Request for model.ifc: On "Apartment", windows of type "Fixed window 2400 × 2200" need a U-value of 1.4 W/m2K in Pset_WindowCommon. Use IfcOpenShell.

First a look at what the model holds.

```python
import ifcopenshell
import ifcopenshell.util.element

model = ifcopenshell.open("model.ifc")
print(model.schema)
storey = next(s for s in model.by_type("IfcBuildingStorey") if s.Name == "Apartment")
windows = [e for e in ifcopenshell.util.element.get_decomposition(storey) if e.is_a("IfcWindow")]
seen = {}
for e in windows:
    element_type = ifcopenshell.util.element.get_type(e)
    key = (element_type.Name if element_type != e and element_type else None, ifcopenshell.util.element.get_pset(e, "Pset_WindowCommon", "ThermalTransmittance"))
    seen[key] = seen.get(key, 0) + 1
for (name, value), count in sorted(seen.items(), key=str):
    print(count, "x", name, "|", value)
```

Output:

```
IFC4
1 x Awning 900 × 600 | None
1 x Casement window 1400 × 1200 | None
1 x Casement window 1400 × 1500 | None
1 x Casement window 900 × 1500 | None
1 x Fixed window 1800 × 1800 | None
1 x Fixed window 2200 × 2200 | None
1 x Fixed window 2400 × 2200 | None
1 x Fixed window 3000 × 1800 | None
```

```python
import ifcopenshell
import ifcopenshell.api.pset
import ifcopenshell.util.element

model = ifcopenshell.open("model.ifc")

storey = next(s for s in model.by_type("IfcBuildingStorey") if s.Name == "Apartment")
windows = [e for e in ifcopenshell.util.element.get_decomposition(storey) if e.is_a("IfcWindow")]

count = 0
for e in windows:
    element_type = ifcopenshell.util.element.get_type(e)
    if element_type in (None, e) or element_type.Name != "Fixed window 2400 × 2200":
        continue
    # add_pset returns the element's existing set when there is one.
    pset = ifcopenshell.api.pset.add_pset(model, product=e, name="Pset_WindowCommon")
    ifcopenshell.api.pset.edit_pset(model, pset=pset, properties={"ThermalTransmittance": 1.4})
    count += 1

print(count, "windows updated")

model.write("model_edited.ifc")
```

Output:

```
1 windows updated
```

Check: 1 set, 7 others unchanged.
